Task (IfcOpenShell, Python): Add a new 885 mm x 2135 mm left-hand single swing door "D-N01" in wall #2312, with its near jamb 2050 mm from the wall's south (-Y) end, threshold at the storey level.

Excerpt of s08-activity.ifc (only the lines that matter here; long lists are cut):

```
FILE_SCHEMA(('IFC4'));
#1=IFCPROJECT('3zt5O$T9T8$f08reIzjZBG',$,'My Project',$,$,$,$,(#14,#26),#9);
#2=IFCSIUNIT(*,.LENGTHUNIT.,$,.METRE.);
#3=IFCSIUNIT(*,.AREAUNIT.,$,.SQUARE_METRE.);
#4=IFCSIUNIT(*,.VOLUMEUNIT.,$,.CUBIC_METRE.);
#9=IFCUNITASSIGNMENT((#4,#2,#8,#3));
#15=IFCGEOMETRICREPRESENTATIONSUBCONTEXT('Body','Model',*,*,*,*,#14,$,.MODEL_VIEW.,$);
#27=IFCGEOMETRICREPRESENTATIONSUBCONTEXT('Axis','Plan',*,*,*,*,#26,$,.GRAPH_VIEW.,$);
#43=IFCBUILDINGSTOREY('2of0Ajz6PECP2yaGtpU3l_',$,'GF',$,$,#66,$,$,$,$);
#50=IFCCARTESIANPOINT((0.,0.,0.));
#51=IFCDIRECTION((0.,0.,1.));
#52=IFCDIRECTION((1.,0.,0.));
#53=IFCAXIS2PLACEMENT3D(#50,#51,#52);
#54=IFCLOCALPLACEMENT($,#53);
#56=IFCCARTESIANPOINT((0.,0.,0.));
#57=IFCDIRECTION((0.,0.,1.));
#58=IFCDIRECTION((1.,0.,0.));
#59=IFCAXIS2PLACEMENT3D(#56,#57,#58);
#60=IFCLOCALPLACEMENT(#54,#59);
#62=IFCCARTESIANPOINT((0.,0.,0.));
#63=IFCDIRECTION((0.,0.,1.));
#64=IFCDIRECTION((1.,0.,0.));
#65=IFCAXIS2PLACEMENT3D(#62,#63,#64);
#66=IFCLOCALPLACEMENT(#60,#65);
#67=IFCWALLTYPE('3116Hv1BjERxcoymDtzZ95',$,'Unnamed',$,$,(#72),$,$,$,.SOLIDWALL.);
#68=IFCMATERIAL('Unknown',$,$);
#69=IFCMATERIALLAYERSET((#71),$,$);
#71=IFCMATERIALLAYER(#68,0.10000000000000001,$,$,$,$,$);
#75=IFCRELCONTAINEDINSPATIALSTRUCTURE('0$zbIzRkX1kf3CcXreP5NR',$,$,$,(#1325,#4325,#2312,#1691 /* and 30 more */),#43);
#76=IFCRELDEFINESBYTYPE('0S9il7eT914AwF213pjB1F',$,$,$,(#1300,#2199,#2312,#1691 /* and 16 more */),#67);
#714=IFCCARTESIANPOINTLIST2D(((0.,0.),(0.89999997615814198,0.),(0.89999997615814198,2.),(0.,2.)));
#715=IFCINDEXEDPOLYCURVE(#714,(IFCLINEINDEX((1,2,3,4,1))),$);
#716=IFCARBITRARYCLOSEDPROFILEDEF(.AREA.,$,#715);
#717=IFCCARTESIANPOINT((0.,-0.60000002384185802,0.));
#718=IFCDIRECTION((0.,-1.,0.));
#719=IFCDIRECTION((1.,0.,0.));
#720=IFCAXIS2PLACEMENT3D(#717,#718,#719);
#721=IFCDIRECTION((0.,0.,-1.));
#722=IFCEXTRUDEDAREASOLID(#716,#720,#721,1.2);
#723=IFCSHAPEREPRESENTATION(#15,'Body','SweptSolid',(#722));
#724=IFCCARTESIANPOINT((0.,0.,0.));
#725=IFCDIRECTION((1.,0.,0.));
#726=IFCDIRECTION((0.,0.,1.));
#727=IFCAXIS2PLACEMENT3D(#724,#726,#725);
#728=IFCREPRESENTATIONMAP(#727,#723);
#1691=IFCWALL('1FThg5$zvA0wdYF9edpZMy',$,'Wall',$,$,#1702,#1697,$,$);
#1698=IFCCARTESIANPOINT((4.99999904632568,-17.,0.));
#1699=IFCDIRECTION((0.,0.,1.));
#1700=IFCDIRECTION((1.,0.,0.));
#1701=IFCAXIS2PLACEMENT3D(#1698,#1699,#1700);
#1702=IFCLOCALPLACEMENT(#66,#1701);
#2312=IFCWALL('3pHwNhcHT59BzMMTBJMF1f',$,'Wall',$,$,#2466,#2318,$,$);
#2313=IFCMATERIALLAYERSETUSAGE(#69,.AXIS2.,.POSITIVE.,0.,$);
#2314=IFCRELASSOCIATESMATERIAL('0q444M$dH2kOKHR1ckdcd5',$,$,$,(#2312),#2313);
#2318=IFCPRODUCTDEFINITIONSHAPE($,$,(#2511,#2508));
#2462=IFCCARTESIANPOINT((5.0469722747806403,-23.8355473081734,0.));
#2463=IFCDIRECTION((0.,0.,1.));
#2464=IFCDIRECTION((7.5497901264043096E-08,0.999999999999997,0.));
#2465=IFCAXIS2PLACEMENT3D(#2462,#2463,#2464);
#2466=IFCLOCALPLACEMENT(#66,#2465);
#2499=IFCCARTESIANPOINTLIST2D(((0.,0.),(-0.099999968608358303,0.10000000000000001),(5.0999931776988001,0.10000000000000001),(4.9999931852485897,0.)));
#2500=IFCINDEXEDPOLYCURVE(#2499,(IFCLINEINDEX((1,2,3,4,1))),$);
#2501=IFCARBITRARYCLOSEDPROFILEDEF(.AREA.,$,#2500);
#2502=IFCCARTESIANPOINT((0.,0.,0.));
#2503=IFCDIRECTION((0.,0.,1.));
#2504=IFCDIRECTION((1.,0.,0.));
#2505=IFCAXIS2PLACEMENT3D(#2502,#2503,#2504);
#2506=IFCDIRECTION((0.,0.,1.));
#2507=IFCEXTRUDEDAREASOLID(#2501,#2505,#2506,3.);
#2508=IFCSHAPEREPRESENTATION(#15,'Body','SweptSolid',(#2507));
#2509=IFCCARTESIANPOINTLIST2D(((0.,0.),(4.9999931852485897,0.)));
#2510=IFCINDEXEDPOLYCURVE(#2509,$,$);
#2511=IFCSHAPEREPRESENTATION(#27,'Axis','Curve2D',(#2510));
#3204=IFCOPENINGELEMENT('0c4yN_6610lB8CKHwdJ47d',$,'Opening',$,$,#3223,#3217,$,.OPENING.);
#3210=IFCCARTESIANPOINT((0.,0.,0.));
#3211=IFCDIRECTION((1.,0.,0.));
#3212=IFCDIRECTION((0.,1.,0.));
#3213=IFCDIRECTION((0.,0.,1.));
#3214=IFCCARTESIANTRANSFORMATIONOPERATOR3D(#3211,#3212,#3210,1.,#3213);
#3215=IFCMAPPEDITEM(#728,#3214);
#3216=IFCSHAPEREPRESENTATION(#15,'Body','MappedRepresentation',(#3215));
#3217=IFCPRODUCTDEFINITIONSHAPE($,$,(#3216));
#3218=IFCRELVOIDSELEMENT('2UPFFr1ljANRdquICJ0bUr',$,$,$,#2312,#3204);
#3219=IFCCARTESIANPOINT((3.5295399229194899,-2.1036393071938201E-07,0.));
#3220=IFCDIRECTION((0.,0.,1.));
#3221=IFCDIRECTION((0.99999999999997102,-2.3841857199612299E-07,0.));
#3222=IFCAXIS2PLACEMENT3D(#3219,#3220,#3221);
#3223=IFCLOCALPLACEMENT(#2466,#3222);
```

```python
import numpy as np
import ifcopenshell
import ifcopenshell.api.feature
import ifcopenshell.api.geometry
import ifcopenshell.api.root
import ifcopenshell.api.spatial
import ifcopenshell.geom
import ifcopenshell.util.element
import ifcopenshell.util.placement
import ifcopenshell.util.representation
import ifcopenshell.util.shape
import ifcopenshell.util.unit

model = ifcopenshell.open("s08-activity.ifc")
unit_scale = ifcopenshell.util.unit.calculate_unit_scale(model)
settings = ifcopenshell.geom.settings()


def volume(element):
    """Net volume in cubic metres, openings subtracted."""
    shape = ifcopenshell.geom.create_shape(settings, element)
    return ifcopenshell.util.shape.get_volume(shape.geometry)


wall = model.by_guid("3pHwNhcHT59BzMMTBJMF1f")
storey = ifcopenshell.util.element.get_container(wall, ifc_class="IfcBuildingStorey")
context = ifcopenshell.util.representation.get_context(model, "Model", "Body", "MODEL_VIEW")
before = volume(wall)

width, height, from_end, sill = 0.885, 2.135, 2.05, 0.0  # metres

# The wall runs along its own X axis, and the end named is its -X end.
wall_shape = ifcopenshell.geom.create_shape(settings, wall)
x, y, z = ifcopenshell.util.shape.get_vertices(wall_shape.geometry).T
start = x.min() + from_end
face, thickness = float(y.min()), float(y.max() - y.min())
wall_matrix = ifcopenshell.util.placement.get_local_placement(wall.ObjectPlacement)
level = ifcopenshell.util.placement.get_local_placement(storey.ObjectPlacement)[2, 3]


def in_wall(x, y):
    """Placement at x, y metres in the wall's axes, at sill height."""
    matrix = wall_matrix.copy()
    matrix[:, 3] = wall_matrix @ np.array([x / unit_scale, y / unit_scale, 0.0, 1.0])
    matrix[2, 3] = level + sill / unit_scale
    return matrix


# Opening: a box that overshoots both wall faces by 50 mm.
opening = ifcopenshell.api.root.create_entity(model, ifc_class="IfcOpeningElement", predefined_type="OPENING")
box = ifcopenshell.api.geometry.add_wall_representation(
    model, context=context, length=width, height=height, thickness=thickness + 0.1
)
ifcopenshell.api.geometry.assign_representation(model, product=opening, representation=box)
ifcopenshell.api.geometry.edit_object_placement(model, product=opening, matrix=in_wall(start, face - 0.05), is_si=False)
ifcopenshell.api.feature.add_feature(model, feature=opening, element=wall)

door = ifcopenshell.api.root.create_entity(model, ifc_class="IfcDoor", name="D-N01", predefined_type="DOOR")
door.OverallWidth, door.OverallHeight = width / unit_scale, height / unit_scale
door.OperationType = "SINGLE_SWING_LEFT"
body = ifcopenshell.api.geometry.add_door_representation(
    model,
    context=context,
    overall_width=door.OverallWidth,
    overall_height=door.OverallHeight,
    operation_type="SINGLE_SWING_LEFT",
    lining_properties={"LiningDepth": thickness / unit_scale, "ThresholdDepth": thickness / unit_scale},
)
ifcopenshell.api.geometry.assign_representation(model, product=door, representation=body)
ifcopenshell.api.spatial.assign_container(model, products=[door], relating_structure=storey)
ifcopenshell.api.feature.add_filling(model, opening=opening, element=door)

# The lining spans the wall, so the door starts at the wall face.
ifcopenshell.api.geometry.edit_object_placement(model, product=door, matrix=in_wall(start, face), is_si=False)

after = volume(wall)

print(f"wall volume {before:.3f} -> {after:.3f} m3")

model.write("s08-activity_v2.ifc")
```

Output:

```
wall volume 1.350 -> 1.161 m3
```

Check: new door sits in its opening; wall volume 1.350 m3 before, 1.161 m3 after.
